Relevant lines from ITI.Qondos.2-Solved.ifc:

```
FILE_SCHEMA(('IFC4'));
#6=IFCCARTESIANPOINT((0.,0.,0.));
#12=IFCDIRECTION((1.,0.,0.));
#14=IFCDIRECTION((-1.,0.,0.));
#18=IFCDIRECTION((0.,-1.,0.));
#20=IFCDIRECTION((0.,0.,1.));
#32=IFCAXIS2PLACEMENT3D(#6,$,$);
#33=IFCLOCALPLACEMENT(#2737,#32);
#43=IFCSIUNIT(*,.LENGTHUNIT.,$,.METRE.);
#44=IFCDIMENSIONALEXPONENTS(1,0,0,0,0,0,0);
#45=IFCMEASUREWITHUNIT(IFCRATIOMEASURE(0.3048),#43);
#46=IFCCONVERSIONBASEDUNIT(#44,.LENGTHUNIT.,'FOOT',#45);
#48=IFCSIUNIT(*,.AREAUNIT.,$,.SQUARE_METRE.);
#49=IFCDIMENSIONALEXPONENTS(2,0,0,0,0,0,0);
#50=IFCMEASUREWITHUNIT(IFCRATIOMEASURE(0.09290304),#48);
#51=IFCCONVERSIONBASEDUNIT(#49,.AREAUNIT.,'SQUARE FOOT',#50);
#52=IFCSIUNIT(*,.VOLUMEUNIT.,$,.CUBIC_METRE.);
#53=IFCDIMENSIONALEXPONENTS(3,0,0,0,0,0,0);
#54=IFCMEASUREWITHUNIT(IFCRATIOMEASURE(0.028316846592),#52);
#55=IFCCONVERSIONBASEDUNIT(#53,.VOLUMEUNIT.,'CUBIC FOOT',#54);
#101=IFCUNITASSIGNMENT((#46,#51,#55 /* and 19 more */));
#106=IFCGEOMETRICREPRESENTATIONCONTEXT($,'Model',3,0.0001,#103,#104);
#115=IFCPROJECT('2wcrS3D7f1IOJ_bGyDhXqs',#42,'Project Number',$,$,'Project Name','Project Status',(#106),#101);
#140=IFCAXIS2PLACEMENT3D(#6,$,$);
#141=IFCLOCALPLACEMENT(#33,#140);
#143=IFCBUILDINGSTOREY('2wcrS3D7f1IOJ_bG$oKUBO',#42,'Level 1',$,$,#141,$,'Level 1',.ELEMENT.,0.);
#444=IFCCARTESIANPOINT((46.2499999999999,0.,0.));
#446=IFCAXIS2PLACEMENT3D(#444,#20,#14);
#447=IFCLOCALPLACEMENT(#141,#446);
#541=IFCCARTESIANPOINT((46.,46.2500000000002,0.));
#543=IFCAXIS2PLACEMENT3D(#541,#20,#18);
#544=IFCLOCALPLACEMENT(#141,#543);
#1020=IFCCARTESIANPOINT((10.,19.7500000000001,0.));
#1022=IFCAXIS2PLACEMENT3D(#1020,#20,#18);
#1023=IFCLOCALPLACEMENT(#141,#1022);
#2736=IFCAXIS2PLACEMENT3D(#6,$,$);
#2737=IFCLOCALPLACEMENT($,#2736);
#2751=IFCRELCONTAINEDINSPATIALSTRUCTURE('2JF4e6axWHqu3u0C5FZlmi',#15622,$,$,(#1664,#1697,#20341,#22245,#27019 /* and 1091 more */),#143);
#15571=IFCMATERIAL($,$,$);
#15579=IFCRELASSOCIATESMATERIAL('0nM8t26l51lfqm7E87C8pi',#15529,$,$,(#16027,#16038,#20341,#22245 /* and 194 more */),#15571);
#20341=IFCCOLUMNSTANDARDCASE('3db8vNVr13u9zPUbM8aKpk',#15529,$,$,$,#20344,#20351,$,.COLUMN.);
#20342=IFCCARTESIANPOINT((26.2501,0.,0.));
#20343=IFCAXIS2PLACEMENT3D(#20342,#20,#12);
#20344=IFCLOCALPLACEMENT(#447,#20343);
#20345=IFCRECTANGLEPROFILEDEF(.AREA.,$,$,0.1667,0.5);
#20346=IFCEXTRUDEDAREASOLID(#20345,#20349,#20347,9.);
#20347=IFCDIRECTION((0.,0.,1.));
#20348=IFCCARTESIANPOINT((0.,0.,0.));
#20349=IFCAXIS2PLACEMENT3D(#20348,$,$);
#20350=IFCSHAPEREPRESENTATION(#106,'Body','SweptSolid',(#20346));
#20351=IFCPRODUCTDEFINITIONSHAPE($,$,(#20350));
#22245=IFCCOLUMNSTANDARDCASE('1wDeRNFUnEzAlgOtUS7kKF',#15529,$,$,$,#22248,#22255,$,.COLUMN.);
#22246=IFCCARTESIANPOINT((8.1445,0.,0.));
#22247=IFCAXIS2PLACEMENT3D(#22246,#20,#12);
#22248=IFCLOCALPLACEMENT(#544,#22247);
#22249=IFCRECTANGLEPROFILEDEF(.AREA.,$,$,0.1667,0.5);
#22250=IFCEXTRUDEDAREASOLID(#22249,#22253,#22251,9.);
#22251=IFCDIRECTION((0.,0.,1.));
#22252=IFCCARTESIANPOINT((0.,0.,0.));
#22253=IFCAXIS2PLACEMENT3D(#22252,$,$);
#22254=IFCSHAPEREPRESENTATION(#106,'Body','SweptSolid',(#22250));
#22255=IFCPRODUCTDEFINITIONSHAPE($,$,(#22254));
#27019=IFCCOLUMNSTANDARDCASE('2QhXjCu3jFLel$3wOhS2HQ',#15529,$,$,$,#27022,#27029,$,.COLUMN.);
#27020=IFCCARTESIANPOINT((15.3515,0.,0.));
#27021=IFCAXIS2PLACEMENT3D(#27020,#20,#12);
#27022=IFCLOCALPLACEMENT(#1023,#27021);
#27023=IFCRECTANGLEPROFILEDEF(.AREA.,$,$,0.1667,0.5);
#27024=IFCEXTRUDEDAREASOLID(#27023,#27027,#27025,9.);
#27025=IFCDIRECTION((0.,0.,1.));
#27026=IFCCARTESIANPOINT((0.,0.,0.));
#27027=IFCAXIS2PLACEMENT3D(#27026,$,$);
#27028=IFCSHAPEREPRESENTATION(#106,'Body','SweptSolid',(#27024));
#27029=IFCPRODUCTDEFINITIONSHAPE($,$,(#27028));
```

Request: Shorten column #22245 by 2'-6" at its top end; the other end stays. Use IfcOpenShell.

```python
import ifcopenshell
import ifcopenshell.util.unit

model = ifcopenshell.open("ITI.Qondos.2-Solved.ifc")
unit_scale = ifcopenshell.util.unit.calculate_unit_scale(model)

member = model.by_guid("1wDeRNFUnEzAlgOtUS7kKF")
change = -30 * 0.0254 / unit_scale

# The extrusion runs towards the end named, so only its depth changes.
body = next(r for r in member.Representation.Representations if r.RepresentationIdentifier == "Body")
solid = body.Items[0]
old_length = solid.Depth
solid.Depth += change

print(f"length {old_length:g} -> {solid.Depth:g}")

model.write("ITI.Qondos.2-Solved_v2.ifc")
```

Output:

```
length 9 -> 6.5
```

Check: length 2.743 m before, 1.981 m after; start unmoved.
